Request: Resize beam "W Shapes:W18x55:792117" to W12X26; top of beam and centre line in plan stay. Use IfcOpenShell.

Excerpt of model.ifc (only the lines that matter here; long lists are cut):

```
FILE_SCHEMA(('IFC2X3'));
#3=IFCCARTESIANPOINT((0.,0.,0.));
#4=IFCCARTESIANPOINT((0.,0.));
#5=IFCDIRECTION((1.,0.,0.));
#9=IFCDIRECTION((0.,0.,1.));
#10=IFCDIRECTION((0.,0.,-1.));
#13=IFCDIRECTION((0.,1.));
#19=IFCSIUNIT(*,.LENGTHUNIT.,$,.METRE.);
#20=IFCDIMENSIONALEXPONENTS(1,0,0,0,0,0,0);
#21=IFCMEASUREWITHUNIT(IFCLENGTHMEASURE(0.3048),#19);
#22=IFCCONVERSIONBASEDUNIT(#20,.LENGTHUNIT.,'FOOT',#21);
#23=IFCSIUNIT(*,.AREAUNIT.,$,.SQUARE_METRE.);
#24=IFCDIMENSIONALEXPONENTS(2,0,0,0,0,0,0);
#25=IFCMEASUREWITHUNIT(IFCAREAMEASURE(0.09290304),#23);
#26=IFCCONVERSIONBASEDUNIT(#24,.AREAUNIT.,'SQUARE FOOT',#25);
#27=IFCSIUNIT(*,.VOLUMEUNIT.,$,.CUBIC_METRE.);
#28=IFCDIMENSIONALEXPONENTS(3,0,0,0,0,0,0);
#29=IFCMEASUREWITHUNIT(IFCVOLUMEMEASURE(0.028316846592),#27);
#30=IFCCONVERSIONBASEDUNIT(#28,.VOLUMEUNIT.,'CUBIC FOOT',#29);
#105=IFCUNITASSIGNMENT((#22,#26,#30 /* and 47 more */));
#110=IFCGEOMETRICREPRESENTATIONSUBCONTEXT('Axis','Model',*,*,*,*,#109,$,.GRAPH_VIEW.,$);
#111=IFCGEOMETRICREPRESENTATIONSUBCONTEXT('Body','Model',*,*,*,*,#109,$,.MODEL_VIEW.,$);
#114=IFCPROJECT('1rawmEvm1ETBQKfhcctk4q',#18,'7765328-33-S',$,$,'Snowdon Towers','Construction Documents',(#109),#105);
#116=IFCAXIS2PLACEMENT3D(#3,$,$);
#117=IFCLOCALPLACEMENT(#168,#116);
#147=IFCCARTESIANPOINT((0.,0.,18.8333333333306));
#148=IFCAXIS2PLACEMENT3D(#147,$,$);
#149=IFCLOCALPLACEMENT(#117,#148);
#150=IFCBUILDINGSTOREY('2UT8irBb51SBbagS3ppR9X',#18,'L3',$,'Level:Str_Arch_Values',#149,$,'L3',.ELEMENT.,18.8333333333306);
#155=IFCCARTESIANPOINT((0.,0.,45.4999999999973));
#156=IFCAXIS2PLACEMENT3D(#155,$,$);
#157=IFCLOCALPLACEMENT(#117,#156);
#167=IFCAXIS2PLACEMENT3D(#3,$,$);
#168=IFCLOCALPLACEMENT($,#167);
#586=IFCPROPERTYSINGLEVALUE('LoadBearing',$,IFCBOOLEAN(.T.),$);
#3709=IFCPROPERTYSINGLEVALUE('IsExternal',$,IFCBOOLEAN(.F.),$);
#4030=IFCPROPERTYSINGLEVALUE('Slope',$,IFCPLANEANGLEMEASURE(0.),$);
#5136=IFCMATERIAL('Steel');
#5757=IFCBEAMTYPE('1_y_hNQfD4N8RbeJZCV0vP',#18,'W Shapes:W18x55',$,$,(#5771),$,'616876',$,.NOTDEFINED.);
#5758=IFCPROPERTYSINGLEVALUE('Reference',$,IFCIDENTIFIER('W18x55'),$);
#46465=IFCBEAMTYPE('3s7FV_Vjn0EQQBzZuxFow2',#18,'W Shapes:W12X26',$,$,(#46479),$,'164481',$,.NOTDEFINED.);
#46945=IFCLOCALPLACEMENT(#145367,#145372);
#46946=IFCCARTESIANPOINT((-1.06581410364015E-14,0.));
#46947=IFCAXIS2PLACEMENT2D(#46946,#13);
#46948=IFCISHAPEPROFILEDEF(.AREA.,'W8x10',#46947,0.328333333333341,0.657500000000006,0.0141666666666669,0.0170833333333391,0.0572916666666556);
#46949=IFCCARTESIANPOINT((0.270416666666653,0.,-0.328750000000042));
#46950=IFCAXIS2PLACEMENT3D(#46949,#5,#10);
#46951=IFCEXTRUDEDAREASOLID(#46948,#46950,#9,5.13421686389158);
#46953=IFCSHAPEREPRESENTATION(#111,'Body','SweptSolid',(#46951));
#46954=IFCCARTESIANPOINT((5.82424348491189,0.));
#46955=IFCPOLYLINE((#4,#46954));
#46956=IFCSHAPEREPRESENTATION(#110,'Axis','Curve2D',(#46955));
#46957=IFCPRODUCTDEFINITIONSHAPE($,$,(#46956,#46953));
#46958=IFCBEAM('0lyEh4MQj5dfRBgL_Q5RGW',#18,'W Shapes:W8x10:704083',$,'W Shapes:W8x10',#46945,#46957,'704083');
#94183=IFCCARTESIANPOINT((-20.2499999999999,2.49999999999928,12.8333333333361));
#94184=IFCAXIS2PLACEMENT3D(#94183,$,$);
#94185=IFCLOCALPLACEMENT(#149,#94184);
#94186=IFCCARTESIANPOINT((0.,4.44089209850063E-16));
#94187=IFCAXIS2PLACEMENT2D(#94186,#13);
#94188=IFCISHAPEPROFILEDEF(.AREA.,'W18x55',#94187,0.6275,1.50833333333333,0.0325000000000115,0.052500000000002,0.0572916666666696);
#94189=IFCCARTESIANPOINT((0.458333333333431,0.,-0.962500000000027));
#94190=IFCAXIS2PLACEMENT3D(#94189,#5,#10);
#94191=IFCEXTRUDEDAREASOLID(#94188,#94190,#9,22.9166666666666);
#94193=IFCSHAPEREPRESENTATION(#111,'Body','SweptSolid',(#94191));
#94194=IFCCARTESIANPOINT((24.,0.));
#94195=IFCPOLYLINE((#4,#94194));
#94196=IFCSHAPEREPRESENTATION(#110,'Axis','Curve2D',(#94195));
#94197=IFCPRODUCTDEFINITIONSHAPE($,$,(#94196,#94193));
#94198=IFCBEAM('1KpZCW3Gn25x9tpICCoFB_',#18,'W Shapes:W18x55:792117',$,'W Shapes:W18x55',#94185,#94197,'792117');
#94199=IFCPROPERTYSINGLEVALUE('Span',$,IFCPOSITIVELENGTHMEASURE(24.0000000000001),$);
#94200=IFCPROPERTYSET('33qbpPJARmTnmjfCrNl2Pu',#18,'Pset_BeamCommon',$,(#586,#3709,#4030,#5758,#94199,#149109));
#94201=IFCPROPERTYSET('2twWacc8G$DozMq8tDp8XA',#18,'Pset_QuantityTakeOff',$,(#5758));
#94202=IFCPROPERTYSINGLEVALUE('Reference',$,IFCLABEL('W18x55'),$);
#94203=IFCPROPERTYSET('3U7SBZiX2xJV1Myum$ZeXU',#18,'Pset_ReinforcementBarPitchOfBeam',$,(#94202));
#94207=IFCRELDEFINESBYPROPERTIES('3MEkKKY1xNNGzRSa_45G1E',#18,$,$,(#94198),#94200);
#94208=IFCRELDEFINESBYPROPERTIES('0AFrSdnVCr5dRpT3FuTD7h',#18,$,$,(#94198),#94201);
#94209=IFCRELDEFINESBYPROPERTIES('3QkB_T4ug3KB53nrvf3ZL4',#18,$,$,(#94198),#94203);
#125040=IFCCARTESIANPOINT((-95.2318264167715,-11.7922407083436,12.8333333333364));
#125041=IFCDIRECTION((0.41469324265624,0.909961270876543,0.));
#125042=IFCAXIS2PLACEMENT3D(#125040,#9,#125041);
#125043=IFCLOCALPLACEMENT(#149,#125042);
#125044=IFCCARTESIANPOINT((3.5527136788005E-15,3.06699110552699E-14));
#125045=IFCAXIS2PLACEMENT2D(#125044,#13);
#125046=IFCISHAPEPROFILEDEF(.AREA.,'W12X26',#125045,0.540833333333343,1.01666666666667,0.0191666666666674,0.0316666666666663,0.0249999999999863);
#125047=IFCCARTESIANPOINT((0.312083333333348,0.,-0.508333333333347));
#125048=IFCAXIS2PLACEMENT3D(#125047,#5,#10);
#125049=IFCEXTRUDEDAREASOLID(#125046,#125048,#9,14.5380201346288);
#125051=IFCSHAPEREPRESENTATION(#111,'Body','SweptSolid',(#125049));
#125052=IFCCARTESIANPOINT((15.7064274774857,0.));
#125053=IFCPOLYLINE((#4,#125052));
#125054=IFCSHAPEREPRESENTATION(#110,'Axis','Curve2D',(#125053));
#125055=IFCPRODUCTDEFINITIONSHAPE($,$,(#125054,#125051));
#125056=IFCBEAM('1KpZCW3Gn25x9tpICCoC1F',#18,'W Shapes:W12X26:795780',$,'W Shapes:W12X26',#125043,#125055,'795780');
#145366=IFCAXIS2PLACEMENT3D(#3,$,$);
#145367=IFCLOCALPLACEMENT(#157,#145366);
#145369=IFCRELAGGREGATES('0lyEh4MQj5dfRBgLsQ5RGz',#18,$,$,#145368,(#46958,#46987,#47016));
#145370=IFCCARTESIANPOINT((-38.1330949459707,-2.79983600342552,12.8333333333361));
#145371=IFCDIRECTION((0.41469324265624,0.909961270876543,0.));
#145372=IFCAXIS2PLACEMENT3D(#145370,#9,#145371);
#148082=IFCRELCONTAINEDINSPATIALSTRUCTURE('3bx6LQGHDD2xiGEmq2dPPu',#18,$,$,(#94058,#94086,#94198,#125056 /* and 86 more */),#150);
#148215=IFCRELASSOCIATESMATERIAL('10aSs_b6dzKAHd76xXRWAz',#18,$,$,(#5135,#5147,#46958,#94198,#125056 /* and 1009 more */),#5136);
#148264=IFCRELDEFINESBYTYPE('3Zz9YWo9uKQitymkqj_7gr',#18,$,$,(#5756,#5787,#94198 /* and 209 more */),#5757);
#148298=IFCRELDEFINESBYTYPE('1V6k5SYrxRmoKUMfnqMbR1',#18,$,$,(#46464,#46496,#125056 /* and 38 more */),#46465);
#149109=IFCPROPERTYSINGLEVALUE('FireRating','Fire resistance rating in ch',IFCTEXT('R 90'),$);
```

```python
import ifcopenshell
import ifcopenshell.api.pset
import ifcopenshell.api.type
import ifcopenshell.util.element
import ifcopenshell.util.representation

model = ifcopenshell.open("model.ifc")

member = model.by_id(94198)
source = next(p for p in model.by_type("IfcIShapeProfileDef") if p.ProfileName == "W12X26")

body = ifcopenshell.util.representation.get_representation(member, "Model", "Body")
solid = body.Items[0]
old_profile = solid.SweptArea

# Copy the section's sizes but keep this member's own profile position.
profile = ifcopenshell.util.element.copy(model, source)
# Profiles are centred, so shift by half the change in depth to hold the top.
shift = (old_profile.OverallDepth - profile.OverallDepth) / 2
x, y = old_profile.Position.Location.Coordinates
up = (-1.0, 0.0)  # upwards, in the solid's own plane
location = model.createIfcCartesianPoint((x + up[0] * shift, y + up[1] * shift))
profile.Position = model.createIfcAxis2Placement2D(location, old_profile.Position.RefDirection)
solid.SweptArea = profile
if not model.get_total_inverses(old_profile):
    ifcopenshell.util.element.remove_deep2(model, old_profile)

new_type = model.by_guid("3s7FV_Vjn0EQQBzZuxFow2")
ifcopenshell.api.type.assign_type(
    model, related_objects=[member], relating_type=new_type, should_map_representations=False
)
member.Name = member.Name.replace("W18x55", "W12X26")
member.ObjectType = "W Shapes:W12X26"
pset = model.by_id(ifcopenshell.util.element.get_pset(member, "Pset_BeamCommon", should_inherit=False)["id"])
ifcopenshell.api.pset.edit_pset(model, pset=pset, properties={"Reference": "W12X26"})
pset = model.by_id(ifcopenshell.util.element.get_pset(member, "Pset_QuantityTakeOff", should_inherit=False)["id"])
ifcopenshell.api.pset.edit_pset(model, pset=pset, properties={"Reference": "W12X26"})
pset = model.by_id(ifcopenshell.util.element.get_pset(member, "Pset_ReinforcementBarPitchOfBeam", should_inherit=False)["id"])
ifcopenshell.api.pset.edit_pset(model, pset=pset, properties={"Reference": "W12X26"})

print(solid.SweptArea)

model.write("model_edited.ifc")
```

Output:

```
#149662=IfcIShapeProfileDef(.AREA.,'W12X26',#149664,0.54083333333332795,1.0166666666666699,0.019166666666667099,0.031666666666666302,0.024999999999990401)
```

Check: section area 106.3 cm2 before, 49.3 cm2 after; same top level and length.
